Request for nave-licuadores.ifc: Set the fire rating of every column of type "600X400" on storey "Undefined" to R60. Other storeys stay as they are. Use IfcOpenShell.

First a look at what the model holds.

```python
import ifcopenshell
import ifcopenshell.util.element

model = ifcopenshell.open("nave-licuadores.ifc")
print(model.schema)
storey = next(s for s in model.by_type("IfcBuildingStorey") if s.Name == "Undefined")
columns = [e for e in ifcopenshell.util.element.get_decomposition(storey) if e.is_a("IfcColumn")]
seen = {}
for e in columns:
    element_type = ifcopenshell.util.element.get_type(e)
    key = (element_type.Name if element_type != e and element_type else None, ifcopenshell.util.element.get_pset(e, "Pset_ColumnCommon", "FireRating"))
    seen[key] = seen.get(key, 0) + 1
for (name, value), count in sorted(seen.items(), key=str):
    print(count, "x", name, "|", value)
```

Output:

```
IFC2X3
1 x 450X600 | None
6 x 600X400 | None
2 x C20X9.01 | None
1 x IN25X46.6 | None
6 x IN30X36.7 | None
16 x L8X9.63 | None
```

```python
import ifcopenshell
import ifcopenshell.api.pset
import ifcopenshell.util.element

model = ifcopenshell.open("nave-licuadores.ifc")

storey = next(s for s in model.by_type("IfcBuildingStorey") if s.Name == "Undefined")
columns = [e for e in ifcopenshell.util.element.get_decomposition(storey) if e.is_a("IfcColumn")]

count = 0
for e in columns:
    element_type = ifcopenshell.util.element.get_type(e)
    if element_type in (None, e) or element_type.Name != "600X400":
        continue
    # add_pset returns the element's existing set when there is one.
    pset = ifcopenshell.api.pset.add_pset(model, product=e, name="Pset_ColumnCommon")
    ifcopenshell.api.pset.edit_pset(model, pset=pset, properties={"FireRating": "R60"})
    count += 1

print(count, "columns updated")

model.write("nave-licuadores_rev.ifc")
```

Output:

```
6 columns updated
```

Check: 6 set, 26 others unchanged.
